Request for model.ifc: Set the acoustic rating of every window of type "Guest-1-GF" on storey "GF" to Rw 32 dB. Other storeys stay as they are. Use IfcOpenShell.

First a look at what the model holds.

```python
import ifcopenshell
import ifcopenshell.util.element

model = ifcopenshell.open("model.ifc")
print(model.schema)
storey = next(s for s in model.by_type("IfcBuildingStorey") if s.Name == "GF")
windows = [e for e in ifcopenshell.util.element.get_decomposition(storey) if e.is_a("IfcWindow")]
seen = {}
for e in windows:
    element_type = ifcopenshell.util.element.get_type(e)
    key = (element_type.Name if element_type != e and element_type else None, ifcopenshell.util.element.get_pset(e, "Pset_WindowCommon", "AcousticRating"))
    seen[key] = seen.get(key, 0) + 1
for (name, value), count in sorted(seen.items(), key=str):
    print(count, "x", name, "|", value)
```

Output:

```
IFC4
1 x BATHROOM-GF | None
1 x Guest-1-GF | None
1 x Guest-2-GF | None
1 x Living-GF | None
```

```python
import ifcopenshell
import ifcopenshell.api.pset
import ifcopenshell.util.element

model = ifcopenshell.open("model.ifc")

storey = next(s for s in model.by_type("IfcBuildingStorey") if s.Name == "GF")
windows = [e for e in ifcopenshell.util.element.get_decomposition(storey) if e.is_a("IfcWindow")]

count = 0
for e in windows:
    element_type = ifcopenshell.util.element.get_type(e)
    if element_type in (None, e) or element_type.Name != "Guest-1-GF":
        continue
    # add_pset returns the element's existing set when there is one.
    pset = ifcopenshell.api.pset.add_pset(model, product=e, name="Pset_WindowCommon")
    ifcopenshell.api.pset.edit_pset(model, pset=pset, properties={"AcousticRating": "Rw 32 dB"})
    count += 1

print(count, "windows updated")

model.write("model_updated.ifc")
```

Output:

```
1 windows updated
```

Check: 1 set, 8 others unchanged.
